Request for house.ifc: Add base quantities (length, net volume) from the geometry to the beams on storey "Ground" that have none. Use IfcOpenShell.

First a look at what the model holds.

```python
import ifcopenshell
import ifcopenshell.util.element
import ifcopenshell.util.unit

model = ifcopenshell.open("house.ifc")
print(model.schema)
for unit_type in ("LENGTHUNIT", "AREAUNIT", "VOLUMEUNIT"):
    print(unit_type, ifcopenshell.util.unit.calculate_unit_scale(model, unit_type))
storey = next(s for s in model.by_type("IfcBuildingStorey") if s.Name == "Ground")
beams = [e for e in ifcopenshell.util.element.get_decomposition(storey) if e.is_a("IfcBeam")]
for e in sorted(beams, key=lambda e: e.id()):
    print(e.id(), e.is_a(), e.Name, list(ifcopenshell.util.element.get_psets(e, qtos_only=True)), sep=" | ")
```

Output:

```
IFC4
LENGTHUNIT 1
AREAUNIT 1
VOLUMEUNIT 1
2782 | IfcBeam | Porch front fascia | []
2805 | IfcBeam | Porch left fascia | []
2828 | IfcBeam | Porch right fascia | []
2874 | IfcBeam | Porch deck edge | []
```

```python
import ifcopenshell
import ifcopenshell.api.pset
import ifcopenshell.geom
import ifcopenshell.util.element
import ifcopenshell.util.shape
import ifcopenshell.util.unit

model = ifcopenshell.open("house.ifc")
unit_scale = ifcopenshell.util.unit.calculate_unit_scale(model)
volume_scale = ifcopenshell.util.unit.calculate_unit_scale(model, "VOLUMEUNIT")
settings = ifcopenshell.geom.settings()

storey = next(s for s in model.by_type("IfcBuildingStorey") if s.Name == "Ground")
beams = [e for e in ifcopenshell.util.element.get_decomposition(storey) if e.is_a("IfcBeam")]

for e in sorted(beams, key=lambda e: e.id()):
    if ifcopenshell.util.element.get_psets(e, qtos_only=True, should_inherit=False):
        continue
    # Geometry comes back in metres, in the element's own axes.
    shape = ifcopenshell.geom.create_shape(settings, e)
    values = {
        "Length": ifcopenshell.util.shape.get_max_xyz(shape.geometry) / unit_scale,
        "NetVolume": ifcopenshell.util.shape.get_volume(shape.geometry) / volume_scale,
    }
    qto = ifcopenshell.api.pset.add_qto(model, product=e, name="Qto_BeamBaseQuantities")
    ifcopenshell.api.pset.edit_qto(model, qto=qto, properties=values)
    print(e.id(), {k: round(v, 3) for k, v in values.items()})

model.write("house_v2.ifc")
```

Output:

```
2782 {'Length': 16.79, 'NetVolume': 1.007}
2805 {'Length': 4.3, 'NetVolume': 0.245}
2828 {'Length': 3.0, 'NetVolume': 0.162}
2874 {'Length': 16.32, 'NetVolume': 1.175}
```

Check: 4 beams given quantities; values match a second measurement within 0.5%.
